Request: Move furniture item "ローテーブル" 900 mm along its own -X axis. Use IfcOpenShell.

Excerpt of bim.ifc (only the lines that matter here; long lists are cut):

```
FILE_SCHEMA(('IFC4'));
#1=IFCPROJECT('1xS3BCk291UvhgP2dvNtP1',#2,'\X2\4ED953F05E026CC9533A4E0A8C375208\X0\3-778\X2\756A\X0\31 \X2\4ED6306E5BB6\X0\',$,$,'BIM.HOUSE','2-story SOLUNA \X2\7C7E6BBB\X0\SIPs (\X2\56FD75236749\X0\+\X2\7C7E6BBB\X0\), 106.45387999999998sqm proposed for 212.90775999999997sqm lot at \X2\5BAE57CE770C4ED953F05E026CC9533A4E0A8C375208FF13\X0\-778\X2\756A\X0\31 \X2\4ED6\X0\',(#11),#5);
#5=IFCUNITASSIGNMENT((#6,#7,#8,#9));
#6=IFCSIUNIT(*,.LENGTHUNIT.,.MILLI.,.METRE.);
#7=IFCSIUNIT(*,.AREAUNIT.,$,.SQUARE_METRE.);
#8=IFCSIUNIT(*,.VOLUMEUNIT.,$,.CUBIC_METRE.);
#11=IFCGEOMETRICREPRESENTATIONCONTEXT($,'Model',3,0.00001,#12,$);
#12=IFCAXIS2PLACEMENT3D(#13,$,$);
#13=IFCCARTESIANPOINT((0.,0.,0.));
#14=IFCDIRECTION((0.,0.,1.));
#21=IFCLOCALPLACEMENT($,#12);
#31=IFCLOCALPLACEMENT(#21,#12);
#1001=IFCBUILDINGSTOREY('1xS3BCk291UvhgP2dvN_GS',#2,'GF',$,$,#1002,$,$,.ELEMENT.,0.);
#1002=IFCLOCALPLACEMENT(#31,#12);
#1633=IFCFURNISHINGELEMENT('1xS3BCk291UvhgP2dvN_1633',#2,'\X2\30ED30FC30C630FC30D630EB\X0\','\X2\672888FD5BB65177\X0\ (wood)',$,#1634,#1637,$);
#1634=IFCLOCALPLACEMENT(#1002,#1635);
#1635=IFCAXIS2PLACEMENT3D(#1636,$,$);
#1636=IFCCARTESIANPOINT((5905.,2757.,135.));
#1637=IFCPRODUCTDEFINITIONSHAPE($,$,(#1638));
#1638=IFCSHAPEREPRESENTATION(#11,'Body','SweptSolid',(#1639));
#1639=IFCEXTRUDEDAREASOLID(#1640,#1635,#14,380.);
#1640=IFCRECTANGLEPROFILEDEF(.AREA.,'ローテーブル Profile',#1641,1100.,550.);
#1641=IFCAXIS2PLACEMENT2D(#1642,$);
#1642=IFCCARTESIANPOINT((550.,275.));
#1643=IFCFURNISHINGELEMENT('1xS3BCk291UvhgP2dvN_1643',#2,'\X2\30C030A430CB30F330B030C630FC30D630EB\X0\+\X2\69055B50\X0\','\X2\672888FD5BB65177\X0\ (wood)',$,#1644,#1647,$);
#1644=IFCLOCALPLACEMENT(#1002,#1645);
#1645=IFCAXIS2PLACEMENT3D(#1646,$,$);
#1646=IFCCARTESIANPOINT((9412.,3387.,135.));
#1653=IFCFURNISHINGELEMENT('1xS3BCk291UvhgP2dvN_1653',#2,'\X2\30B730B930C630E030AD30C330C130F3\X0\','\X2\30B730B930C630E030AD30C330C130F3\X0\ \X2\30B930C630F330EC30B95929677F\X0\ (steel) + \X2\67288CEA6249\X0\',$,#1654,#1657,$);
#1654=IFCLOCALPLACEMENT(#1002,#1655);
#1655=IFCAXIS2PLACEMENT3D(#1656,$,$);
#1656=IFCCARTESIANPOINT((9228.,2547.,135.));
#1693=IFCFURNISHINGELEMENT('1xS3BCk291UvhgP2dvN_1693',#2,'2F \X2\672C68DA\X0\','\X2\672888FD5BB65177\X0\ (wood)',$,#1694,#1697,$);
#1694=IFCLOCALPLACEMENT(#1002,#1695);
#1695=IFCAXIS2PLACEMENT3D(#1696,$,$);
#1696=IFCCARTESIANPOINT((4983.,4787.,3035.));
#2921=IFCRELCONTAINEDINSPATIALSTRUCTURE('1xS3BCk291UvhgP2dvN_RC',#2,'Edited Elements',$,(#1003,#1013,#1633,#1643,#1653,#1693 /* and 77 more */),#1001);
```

```python
import ifcopenshell
import ifcopenshell.api.geometry
import ifcopenshell.util.placement
import ifcopenshell.util.unit

model = ifcopenshell.open("bim.ifc")
unit_scale = ifcopenshell.util.unit.calculate_unit_scale(model)

item = model.by_guid("1xS3BCk291UvhgP2dvN_1633")
matrix = ifcopenshell.util.placement.get_local_placement(item.ObjectPlacement)
matrix[:3, 3] -= matrix[:3, 0] * 0.9 / unit_scale
ifcopenshell.api.geometry.edit_object_placement(model, product=item, matrix=matrix, is_si=False)

print(ifcopenshell.util.placement.get_local_placement(item.ObjectPlacement).round(3) + 0.0)

model.write("bim-out.ifc")
```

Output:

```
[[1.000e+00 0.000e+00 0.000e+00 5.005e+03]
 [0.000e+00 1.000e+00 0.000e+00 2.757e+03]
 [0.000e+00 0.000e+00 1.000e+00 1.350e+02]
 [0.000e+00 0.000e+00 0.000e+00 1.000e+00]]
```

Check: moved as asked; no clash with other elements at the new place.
